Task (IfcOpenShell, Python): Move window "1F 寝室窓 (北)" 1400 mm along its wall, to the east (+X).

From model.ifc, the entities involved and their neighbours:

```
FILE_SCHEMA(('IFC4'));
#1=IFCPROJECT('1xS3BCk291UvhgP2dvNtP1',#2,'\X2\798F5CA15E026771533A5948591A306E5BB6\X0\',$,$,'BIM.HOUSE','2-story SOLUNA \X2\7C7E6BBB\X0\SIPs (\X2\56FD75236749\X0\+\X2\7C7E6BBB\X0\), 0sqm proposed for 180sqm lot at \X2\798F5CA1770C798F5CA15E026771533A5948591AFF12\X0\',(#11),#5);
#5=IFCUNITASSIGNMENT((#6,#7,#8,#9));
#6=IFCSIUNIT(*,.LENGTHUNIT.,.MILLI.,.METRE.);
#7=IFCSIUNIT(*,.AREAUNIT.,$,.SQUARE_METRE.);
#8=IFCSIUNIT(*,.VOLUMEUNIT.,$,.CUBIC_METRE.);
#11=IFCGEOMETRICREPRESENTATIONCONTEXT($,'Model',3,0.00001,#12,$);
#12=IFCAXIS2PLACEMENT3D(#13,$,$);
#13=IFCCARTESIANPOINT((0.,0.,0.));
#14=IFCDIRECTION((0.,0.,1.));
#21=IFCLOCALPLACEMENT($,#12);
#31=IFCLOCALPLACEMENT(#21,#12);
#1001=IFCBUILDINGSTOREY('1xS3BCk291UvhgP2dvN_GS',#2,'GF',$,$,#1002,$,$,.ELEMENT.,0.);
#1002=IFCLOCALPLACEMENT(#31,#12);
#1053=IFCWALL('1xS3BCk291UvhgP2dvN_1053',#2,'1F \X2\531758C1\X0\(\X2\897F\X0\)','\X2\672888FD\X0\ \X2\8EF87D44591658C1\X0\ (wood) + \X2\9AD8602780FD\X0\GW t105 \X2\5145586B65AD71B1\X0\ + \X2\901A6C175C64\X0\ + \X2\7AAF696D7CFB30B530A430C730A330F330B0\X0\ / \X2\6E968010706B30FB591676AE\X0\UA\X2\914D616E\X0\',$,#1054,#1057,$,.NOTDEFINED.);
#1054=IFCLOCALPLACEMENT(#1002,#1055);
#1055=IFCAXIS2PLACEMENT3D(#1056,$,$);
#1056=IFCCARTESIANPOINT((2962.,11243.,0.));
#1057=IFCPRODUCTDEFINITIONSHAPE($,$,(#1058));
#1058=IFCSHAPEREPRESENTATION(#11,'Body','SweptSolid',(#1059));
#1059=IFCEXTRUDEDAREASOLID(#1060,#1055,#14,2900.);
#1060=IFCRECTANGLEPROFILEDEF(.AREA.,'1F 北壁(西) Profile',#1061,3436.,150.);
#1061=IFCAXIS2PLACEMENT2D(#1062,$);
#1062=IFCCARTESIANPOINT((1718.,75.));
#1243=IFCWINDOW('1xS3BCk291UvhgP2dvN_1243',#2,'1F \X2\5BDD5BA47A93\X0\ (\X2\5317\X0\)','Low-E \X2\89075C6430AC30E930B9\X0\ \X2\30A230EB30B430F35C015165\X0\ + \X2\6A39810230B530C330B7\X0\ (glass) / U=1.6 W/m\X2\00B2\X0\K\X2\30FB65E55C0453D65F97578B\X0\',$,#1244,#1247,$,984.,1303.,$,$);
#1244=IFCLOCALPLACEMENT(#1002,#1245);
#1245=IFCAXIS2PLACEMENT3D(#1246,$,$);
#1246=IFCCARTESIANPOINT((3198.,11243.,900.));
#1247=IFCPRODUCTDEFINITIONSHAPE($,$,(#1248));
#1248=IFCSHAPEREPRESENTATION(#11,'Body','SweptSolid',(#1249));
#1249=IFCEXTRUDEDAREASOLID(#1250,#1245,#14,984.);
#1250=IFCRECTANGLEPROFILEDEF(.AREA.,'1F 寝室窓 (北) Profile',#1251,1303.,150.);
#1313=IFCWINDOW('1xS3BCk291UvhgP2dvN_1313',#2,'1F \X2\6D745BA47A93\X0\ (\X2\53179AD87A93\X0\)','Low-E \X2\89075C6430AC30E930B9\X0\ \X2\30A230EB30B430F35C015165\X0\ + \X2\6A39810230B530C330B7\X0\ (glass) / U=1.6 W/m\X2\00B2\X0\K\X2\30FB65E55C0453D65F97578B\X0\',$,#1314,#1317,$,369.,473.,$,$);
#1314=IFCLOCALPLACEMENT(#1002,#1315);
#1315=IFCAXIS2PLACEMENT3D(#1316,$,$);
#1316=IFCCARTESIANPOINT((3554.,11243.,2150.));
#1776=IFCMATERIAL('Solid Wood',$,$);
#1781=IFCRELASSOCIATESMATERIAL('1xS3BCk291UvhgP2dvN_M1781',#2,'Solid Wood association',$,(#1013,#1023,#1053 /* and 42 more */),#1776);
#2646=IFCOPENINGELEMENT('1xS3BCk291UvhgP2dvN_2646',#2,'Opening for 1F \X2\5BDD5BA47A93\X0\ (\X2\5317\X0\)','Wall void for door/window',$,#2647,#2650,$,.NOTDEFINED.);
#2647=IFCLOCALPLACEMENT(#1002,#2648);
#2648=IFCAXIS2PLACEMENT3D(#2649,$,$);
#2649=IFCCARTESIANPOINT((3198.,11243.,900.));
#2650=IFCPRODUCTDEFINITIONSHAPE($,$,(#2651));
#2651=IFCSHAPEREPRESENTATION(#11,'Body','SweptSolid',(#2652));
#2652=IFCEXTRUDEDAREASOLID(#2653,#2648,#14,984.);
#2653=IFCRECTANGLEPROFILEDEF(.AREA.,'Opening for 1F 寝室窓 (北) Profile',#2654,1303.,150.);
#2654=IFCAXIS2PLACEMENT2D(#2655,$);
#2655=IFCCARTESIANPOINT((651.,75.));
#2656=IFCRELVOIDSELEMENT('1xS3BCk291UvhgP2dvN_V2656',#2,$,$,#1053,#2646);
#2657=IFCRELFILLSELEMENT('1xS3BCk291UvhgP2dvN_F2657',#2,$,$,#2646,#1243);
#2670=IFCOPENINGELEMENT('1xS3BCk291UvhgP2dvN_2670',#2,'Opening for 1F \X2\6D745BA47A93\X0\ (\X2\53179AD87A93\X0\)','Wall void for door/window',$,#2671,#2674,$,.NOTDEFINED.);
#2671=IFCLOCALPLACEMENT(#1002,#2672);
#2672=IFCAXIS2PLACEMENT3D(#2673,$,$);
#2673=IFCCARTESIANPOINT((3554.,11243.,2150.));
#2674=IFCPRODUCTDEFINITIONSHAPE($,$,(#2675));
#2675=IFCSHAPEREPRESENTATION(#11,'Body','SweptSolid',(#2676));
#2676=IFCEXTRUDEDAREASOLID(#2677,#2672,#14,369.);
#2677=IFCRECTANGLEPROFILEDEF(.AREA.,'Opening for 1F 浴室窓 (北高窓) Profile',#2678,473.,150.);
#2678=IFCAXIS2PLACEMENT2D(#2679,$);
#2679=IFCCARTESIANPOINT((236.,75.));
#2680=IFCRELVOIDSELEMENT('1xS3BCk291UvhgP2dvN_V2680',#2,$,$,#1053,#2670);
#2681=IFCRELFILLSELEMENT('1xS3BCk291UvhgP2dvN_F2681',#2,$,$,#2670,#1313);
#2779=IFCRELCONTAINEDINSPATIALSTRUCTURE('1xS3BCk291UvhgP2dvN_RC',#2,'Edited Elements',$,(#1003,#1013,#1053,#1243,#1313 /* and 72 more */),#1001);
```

```python
import ifcopenshell
import ifcopenshell.api.geometry
import ifcopenshell.util.placement

model = ifcopenshell.open("model.ifc")

window = model.by_id(1243)
opening = window.FillsVoids[0].RelatingOpeningElement
wall = opening.VoidsElements[0].RelatingBuildingElement

wall_matrix = ifcopenshell.util.placement.get_local_placement(wall.ObjectPlacement)
shift = wall_matrix[:3, 0] * 1400.0
before = ifcopenshell.util.placement.get_local_placement(window.ObjectPlacement)[:3, 3].copy()

# The window is not placed relative to its opening, so move both.
for product in (opening, window):
    matrix = ifcopenshell.util.placement.get_local_placement(product.ObjectPlacement)
    matrix[:3, 3] += shift
    ifcopenshell.api.geometry.edit_object_placement(model, product=product, matrix=matrix, is_si=False)

after = ifcopenshell.util.placement.get_local_placement(window.ObjectPlacement)[:3, 3]
print("window moved by", (after - before).round(3) + 0.0)

model.write("model_edited.ifc")
```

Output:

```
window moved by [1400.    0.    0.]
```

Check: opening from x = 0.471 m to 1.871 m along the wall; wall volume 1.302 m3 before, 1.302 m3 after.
